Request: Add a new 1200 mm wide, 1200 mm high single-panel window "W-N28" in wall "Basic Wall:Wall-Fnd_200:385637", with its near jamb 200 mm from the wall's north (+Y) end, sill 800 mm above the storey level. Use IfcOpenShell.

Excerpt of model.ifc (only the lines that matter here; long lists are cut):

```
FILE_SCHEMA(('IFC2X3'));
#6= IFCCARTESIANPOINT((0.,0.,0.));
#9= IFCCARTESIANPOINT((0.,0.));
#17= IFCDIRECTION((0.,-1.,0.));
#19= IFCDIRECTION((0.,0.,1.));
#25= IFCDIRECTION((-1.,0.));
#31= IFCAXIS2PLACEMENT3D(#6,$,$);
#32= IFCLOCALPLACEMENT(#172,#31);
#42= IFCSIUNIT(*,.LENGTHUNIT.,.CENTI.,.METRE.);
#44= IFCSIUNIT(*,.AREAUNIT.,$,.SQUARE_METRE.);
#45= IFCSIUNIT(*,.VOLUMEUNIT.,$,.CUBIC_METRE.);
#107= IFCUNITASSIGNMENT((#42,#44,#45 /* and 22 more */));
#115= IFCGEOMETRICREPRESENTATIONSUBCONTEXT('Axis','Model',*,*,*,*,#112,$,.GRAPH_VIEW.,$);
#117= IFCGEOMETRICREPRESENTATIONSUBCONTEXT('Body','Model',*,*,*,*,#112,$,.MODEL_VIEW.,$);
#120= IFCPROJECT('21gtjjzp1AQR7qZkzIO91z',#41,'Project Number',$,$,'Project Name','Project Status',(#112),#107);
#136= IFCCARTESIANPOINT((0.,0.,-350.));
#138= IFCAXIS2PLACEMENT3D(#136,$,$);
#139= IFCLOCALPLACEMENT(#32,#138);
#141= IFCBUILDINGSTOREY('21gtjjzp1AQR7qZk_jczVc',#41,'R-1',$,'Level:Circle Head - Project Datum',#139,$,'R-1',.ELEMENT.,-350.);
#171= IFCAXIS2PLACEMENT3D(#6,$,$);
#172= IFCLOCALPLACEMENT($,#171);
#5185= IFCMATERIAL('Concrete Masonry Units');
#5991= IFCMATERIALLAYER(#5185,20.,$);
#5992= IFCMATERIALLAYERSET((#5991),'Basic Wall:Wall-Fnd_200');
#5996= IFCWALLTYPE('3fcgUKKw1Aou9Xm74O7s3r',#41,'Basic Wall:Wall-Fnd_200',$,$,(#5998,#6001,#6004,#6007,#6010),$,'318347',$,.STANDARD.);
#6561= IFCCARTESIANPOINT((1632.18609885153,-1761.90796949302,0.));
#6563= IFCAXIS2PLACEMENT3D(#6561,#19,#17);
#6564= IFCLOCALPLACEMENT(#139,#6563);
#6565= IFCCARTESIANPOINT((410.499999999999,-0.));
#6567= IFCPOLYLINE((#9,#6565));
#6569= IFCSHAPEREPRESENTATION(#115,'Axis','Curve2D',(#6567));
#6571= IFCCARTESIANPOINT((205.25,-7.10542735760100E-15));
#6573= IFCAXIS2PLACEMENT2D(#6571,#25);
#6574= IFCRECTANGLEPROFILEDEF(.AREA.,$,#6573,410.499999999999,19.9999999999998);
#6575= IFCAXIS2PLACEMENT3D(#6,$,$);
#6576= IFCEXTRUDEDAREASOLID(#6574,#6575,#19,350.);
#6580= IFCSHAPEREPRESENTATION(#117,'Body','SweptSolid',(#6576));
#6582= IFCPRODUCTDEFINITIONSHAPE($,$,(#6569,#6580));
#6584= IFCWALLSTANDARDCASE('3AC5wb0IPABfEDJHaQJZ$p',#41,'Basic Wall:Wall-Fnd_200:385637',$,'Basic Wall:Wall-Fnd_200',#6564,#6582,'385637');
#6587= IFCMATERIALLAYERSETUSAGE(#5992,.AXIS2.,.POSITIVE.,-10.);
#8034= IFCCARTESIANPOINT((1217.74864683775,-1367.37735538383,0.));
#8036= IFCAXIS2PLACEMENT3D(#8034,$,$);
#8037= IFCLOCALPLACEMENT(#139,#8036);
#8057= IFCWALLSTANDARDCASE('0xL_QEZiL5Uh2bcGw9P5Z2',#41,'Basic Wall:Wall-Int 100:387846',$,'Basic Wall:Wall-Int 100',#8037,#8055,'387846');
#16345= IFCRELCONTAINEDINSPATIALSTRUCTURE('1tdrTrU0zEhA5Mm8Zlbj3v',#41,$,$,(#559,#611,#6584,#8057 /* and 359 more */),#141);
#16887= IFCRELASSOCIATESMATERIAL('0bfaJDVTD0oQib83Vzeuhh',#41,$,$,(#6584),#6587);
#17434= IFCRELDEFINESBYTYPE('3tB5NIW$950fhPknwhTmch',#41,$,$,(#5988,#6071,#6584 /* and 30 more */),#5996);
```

```python
import numpy as np
import ifcopenshell
import ifcopenshell.api.feature
import ifcopenshell.api.geometry
import ifcopenshell.api.root
import ifcopenshell.api.spatial
import ifcopenshell.api.type
import ifcopenshell.geom
import ifcopenshell.util.element
import ifcopenshell.util.placement
import ifcopenshell.util.representation
import ifcopenshell.util.shape
import ifcopenshell.util.unit

model = ifcopenshell.open("model.ifc")
unit_scale = ifcopenshell.util.unit.calculate_unit_scale(model)
settings = ifcopenshell.geom.settings()


def volume(element):
    """Net volume in cubic metres, openings subtracted."""
    shape = ifcopenshell.geom.create_shape(settings, element)
    return ifcopenshell.util.shape.get_volume(shape.geometry)


wall = model.by_guid("3AC5wb0IPABfEDJHaQJZ$p")
storey = ifcopenshell.util.element.get_container(wall, ifc_class="IfcBuildingStorey")
context = ifcopenshell.util.representation.get_context(model, "Model", "Body", "MODEL_VIEW")
before = volume(wall)

width, height, from_end, sill = 1.2, 1.2, 0.2, 0.8  # metres

# The wall runs along its own X axis, and the end named is its -X end.
wall_shape = ifcopenshell.geom.create_shape(settings, wall)
x, y, z = ifcopenshell.util.shape.get_vertices(wall_shape.geometry).T
start = x.min() + from_end
face, thickness = float(y.min()), float(y.max() - y.min())
wall_matrix = ifcopenshell.util.placement.get_local_placement(wall.ObjectPlacement)
level = ifcopenshell.util.placement.get_local_placement(storey.ObjectPlacement)[2, 3]


def in_wall(x, y):
    """Placement at x, y metres in the wall's axes, at sill height."""
    matrix = wall_matrix.copy()
    matrix[:, 3] = wall_matrix @ np.array([x / unit_scale, y / unit_scale, 0.0, 1.0])
    matrix[2, 3] = level + sill / unit_scale
    return matrix


# Opening: a box that overshoots both wall faces by 50 mm.
opening = ifcopenshell.api.root.create_entity(model, ifc_class="IfcOpeningElement")
box = ifcopenshell.api.geometry.add_wall_representation(
    model, context=context, length=width, height=height, thickness=thickness + 0.1
)
ifcopenshell.api.geometry.assign_representation(model, product=opening, representation=box)
ifcopenshell.api.geometry.edit_object_placement(model, product=opening, matrix=in_wall(start, face - 0.05), is_si=False)
ifcopenshell.api.feature.add_feature(model, feature=opening, element=wall)

window = ifcopenshell.api.root.create_entity(model, ifc_class="IfcWindow", name="W-N28")
window.OverallWidth, window.OverallHeight = width / unit_scale, height / unit_scale
body = ifcopenshell.api.geometry.add_window_representation(
    model,
    context=context,
    overall_width=window.OverallWidth,
    overall_height=window.OverallHeight,
    partition_type="SINGLE_PANEL",
)
ifcopenshell.api.geometry.assign_representation(model, product=window, representation=body)
ifcopenshell.api.spatial.assign_container(model, products=[window], relating_structure=storey)
fills = ifcopenshell.api.feature.add_filling(model, opening=opening, element=window)
fills.OwnerHistory = window.OwnerHistory  # required in IFC2X3

# IFC2X3 keeps the operation on the window style.
style = ifcopenshell.api.root.create_entity(model, ifc_class="IfcWindowStyle", name="W-N28")
style.OperationType, style.ConstructionType = "SINGLE_PANEL", "NOTDEFINED"
style.ParameterTakesPrecedence = style.Sizeable = False
ifcopenshell.api.type.assign_type(model, related_objects=[window], relating_type=style)

# Centre the window in the wall's thickness.
ifcopenshell.api.geometry.edit_object_placement(model, product=window, matrix=in_wall(start, face), is_si=False)
window_shape = ifcopenshell.geom.create_shape(settings, window)
depth = ifcopenshell.util.shape.get_vertices(window_shape.geometry)[:, 1]
offset = face + thickness / 2 - (depth.min() + depth.max()) / 2
ifcopenshell.api.geometry.edit_object_placement(model, product=window, matrix=in_wall(start, offset), is_si=False)

after = volume(wall)

print(f"wall volume {before:.3f} -> {after:.3f} m3")

model.write("model_updated.ifc")
```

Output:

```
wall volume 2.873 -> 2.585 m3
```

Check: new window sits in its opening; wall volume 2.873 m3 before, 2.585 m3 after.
